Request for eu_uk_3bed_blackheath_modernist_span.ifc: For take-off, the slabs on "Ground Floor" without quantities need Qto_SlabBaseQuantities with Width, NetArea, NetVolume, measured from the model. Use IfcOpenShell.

First a look at what the model holds.

```python
import ifcopenshell
import ifcopenshell.util.element
import ifcopenshell.util.unit

model = ifcopenshell.open("eu_uk_3bed_blackheath_modernist_span.ifc")
print(model.schema)
for unit_type in ("LENGTHUNIT", "AREAUNIT", "VOLUMEUNIT"):
    print(unit_type, ifcopenshell.util.unit.calculate_unit_scale(model, unit_type))
storey = next(s for s in model.by_type("IfcBuildingStorey") if s.Name == "Ground Floor")
slabs = [e for e in ifcopenshell.util.element.get_decomposition(storey) if e.is_a("IfcSlab")]
for e in sorted(slabs, key=lambda e: e.id()):
    print(e.id(), e.is_a(), e.Name, list(ifcopenshell.util.element.get_psets(e, qtos_only=True)), sep=" | ")
```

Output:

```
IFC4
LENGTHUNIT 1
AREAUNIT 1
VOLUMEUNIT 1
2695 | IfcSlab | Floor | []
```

```python
import ifcopenshell
import ifcopenshell.api.pset
import ifcopenshell.geom
import ifcopenshell.util.element
import ifcopenshell.util.shape
import ifcopenshell.util.unit

model = ifcopenshell.open("eu_uk_3bed_blackheath_modernist_span.ifc")
unit_scale = ifcopenshell.util.unit.calculate_unit_scale(model)
area_scale = ifcopenshell.util.unit.calculate_unit_scale(model, "AREAUNIT")
volume_scale = ifcopenshell.util.unit.calculate_unit_scale(model, "VOLUMEUNIT")
settings = ifcopenshell.geom.settings()

storey = next(s for s in model.by_type("IfcBuildingStorey") if s.Name == "Ground Floor")
slabs = [e for e in ifcopenshell.util.element.get_decomposition(storey) if e.is_a("IfcSlab")]

for e in sorted(slabs, key=lambda e: e.id()):
    if ifcopenshell.util.element.get_psets(e, qtos_only=True, should_inherit=False):
        continue
    # Geometry comes back in metres, in the element's own axes.
    shape = ifcopenshell.geom.create_shape(settings, e)
    values = {
        "Width": ifcopenshell.util.shape.get_z(shape.geometry) / unit_scale,
        "NetArea": ifcopenshell.util.shape.get_footprint_area(shape.geometry) / area_scale,
        "NetVolume": ifcopenshell.util.shape.get_volume(shape.geometry) / volume_scale,
    }
    qto = ifcopenshell.api.pset.add_qto(model, product=e, name="Qto_SlabBaseQuantities")
    ifcopenshell.api.pset.edit_qto(model, qto=qto, properties=values)
    print(e.id(), {k: round(v, 3) for k, v in values.items()})

model.write("eu_uk_3bed_blackheath_modernist_span-out.ifc")
```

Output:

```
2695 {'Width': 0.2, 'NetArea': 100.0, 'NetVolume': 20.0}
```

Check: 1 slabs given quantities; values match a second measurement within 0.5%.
